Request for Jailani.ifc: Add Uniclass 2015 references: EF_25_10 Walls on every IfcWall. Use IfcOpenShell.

First a look at what the model holds.

```python
import ifcopenshell

model = ifcopenshell.open("Jailani.ifc")
print(model.schema)
print("classifications:", [c.Name for c in model.by_type("IfcClassification")])
for ifc_class in ("IfcDoor", "IfcRoof", "IfcStair", "IfcWall", "IfcWindow"):
    print(ifc_class, len(model.by_type(ifc_class)))
```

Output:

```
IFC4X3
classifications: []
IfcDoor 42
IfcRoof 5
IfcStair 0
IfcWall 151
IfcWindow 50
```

```python
import ifcopenshell
import ifcopenshell.api.classification

model = ifcopenshell.open("Jailani.ifc")

system = ifcopenshell.api.classification.add_classification(model, classification="Uniclass 2015")

codes = {
    "IfcWall": ("EF_25_10", "Walls"),
}
for ifc_class, (code, name) in codes.items():
    products = model.by_type(ifc_class)
    ifcopenshell.api.classification.add_reference(
        model, products=products, classification=system, identification=code, name=name
    )
    print(code, len(products))

model.write("Jailani_edited.ifc")
```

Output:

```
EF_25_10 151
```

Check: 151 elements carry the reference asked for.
